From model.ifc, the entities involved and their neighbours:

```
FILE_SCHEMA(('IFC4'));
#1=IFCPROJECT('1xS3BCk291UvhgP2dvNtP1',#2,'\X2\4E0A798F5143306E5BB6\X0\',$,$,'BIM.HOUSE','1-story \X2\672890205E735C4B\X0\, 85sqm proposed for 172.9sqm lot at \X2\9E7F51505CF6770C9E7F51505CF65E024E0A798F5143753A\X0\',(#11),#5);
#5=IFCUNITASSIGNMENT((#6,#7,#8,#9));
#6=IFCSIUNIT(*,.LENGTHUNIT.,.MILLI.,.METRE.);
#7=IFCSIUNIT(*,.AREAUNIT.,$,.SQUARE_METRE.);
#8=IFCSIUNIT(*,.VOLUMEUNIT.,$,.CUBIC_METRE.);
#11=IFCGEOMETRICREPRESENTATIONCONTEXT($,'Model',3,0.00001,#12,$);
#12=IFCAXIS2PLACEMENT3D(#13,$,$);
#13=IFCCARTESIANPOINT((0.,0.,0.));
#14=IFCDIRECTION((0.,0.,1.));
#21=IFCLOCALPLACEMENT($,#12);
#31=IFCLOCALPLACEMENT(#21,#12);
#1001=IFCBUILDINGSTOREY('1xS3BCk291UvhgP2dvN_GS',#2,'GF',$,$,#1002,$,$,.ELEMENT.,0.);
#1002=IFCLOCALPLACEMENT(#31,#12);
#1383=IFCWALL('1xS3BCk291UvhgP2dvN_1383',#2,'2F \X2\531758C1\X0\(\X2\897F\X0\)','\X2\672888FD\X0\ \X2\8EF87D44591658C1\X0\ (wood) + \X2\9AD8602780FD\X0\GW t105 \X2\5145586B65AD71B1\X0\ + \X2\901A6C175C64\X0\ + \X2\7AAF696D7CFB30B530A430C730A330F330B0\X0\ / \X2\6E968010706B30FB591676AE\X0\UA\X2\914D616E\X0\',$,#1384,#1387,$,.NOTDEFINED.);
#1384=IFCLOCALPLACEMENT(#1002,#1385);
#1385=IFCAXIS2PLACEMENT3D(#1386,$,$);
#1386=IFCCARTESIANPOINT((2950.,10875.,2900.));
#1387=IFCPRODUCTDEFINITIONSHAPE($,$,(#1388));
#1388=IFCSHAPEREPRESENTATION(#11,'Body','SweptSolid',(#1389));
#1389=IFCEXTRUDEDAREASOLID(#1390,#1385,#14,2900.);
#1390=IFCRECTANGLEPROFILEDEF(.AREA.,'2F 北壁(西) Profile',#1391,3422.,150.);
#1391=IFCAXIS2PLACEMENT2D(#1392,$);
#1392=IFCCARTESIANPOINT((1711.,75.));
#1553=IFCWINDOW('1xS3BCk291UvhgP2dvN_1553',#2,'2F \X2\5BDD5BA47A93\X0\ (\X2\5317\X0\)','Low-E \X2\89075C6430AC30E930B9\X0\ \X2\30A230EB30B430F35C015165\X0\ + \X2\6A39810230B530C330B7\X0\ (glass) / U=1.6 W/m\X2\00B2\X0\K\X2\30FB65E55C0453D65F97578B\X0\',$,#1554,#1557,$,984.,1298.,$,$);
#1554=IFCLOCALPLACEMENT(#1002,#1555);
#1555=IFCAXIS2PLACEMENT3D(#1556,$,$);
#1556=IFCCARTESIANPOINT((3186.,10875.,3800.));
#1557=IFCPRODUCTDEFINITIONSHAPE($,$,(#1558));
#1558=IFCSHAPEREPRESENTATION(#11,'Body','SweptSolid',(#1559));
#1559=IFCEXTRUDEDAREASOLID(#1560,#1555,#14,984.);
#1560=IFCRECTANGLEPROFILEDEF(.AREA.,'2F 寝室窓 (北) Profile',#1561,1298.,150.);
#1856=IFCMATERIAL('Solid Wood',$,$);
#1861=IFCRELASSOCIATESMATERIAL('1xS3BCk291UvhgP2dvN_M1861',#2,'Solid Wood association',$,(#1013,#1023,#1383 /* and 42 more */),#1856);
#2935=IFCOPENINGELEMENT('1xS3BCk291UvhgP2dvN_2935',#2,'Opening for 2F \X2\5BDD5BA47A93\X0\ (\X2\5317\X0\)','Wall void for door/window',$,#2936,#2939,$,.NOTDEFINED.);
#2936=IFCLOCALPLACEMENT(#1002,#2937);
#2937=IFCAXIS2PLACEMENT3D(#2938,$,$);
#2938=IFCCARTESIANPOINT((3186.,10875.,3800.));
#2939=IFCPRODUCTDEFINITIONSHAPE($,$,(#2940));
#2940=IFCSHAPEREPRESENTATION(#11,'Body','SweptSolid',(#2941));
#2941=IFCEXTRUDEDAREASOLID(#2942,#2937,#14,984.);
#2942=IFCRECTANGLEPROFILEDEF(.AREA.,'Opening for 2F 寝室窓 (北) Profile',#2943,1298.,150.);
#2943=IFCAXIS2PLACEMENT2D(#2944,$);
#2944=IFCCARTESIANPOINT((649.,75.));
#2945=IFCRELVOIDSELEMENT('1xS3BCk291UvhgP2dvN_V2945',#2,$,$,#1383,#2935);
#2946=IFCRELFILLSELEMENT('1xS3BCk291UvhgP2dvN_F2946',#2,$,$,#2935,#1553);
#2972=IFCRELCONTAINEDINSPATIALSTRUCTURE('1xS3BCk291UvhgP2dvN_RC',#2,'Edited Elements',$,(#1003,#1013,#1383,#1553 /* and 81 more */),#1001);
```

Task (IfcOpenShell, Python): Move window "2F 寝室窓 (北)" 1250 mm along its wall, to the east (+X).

```python
import ifcopenshell
import ifcopenshell.api.geometry
import ifcopenshell.util.placement

model = ifcopenshell.open("model.ifc")

window = model.by_id(1553)
opening = window.FillsVoids[0].RelatingOpeningElement
wall = opening.VoidsElements[0].RelatingBuildingElement

wall_matrix = ifcopenshell.util.placement.get_local_placement(wall.ObjectPlacement)
shift = wall_matrix[:3, 0] * 1250.0
before = ifcopenshell.util.placement.get_local_placement(window.ObjectPlacement)[:3, 3].copy()

# The window is not placed relative to its opening, so move both.
for product in (opening, window):
    matrix = ifcopenshell.util.placement.get_local_placement(product.ObjectPlacement)
    matrix[:3, 3] += shift
    ifcopenshell.api.geometry.edit_object_placement(model, product=product, matrix=matrix, is_si=False)

after = ifcopenshell.util.placement.get_local_placement(window.ObjectPlacement)[:3, 3]
print("window moved by", (after - before).round(3) + 0.0)

model.write("model_rev.ifc")
```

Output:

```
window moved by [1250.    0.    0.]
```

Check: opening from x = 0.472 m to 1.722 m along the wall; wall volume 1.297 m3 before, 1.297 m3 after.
